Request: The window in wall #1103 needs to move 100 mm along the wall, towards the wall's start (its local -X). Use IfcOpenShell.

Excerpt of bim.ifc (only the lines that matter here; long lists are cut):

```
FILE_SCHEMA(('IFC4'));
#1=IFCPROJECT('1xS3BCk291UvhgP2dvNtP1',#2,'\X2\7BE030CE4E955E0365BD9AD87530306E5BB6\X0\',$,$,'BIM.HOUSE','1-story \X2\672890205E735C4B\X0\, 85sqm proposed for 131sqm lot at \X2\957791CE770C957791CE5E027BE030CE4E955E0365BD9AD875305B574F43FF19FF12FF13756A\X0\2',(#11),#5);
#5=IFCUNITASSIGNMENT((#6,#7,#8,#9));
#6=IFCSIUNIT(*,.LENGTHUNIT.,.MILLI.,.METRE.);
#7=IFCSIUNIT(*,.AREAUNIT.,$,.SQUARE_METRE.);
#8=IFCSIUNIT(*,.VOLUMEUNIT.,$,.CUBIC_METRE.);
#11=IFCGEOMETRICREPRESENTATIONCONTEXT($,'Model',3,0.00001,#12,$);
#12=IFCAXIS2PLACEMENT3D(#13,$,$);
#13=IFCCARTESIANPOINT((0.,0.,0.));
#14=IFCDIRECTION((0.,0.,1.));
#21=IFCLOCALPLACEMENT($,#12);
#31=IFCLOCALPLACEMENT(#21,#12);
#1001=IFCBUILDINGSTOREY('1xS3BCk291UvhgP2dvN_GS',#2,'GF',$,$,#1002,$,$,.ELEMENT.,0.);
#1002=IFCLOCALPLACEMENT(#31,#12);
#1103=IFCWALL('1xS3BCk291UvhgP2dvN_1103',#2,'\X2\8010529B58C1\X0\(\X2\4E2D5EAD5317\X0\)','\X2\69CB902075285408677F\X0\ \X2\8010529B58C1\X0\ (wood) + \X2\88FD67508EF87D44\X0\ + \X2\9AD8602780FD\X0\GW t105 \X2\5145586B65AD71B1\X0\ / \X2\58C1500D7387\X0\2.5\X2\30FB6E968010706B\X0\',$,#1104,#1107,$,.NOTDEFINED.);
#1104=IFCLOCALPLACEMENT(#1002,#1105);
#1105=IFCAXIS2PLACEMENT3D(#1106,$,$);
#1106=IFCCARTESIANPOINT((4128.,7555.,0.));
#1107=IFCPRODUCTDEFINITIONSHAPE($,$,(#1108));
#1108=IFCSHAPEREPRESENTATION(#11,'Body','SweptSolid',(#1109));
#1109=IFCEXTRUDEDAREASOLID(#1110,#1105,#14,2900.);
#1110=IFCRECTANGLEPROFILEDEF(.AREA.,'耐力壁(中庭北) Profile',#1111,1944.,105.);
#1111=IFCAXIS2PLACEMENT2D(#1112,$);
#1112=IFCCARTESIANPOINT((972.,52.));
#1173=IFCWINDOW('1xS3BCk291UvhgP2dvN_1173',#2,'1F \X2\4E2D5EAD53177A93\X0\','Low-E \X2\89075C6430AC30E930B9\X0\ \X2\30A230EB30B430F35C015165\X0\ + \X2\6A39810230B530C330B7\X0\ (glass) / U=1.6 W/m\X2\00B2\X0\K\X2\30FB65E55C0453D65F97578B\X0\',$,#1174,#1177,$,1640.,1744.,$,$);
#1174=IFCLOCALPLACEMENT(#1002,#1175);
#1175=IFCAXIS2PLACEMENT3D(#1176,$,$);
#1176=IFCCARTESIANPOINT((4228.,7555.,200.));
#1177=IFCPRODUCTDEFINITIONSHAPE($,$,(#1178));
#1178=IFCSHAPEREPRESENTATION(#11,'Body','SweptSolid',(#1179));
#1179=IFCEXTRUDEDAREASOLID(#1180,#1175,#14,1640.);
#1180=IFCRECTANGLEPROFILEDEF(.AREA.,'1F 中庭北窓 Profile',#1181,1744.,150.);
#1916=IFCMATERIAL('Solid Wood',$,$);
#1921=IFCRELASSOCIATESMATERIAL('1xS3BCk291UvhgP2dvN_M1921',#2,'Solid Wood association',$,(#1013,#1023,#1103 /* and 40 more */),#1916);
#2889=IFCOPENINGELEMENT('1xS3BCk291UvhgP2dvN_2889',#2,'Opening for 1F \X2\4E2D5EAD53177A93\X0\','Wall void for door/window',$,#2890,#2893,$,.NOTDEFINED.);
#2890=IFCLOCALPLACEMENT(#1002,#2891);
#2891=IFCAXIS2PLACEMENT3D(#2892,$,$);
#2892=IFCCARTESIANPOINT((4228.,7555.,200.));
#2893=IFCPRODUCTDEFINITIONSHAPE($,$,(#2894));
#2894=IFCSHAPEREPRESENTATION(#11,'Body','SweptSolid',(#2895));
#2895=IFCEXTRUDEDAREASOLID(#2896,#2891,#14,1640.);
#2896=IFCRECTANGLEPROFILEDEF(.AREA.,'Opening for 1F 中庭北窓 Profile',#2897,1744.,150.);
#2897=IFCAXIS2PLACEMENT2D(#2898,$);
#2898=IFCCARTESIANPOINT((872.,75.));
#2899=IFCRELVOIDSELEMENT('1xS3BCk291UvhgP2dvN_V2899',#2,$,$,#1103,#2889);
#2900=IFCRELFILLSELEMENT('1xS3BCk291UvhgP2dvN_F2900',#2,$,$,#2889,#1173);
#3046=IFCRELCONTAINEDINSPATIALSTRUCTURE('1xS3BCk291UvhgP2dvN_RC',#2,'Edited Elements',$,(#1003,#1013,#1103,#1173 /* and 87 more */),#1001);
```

```python
import ifcopenshell
import ifcopenshell.api.geometry
import ifcopenshell.util.placement
import ifcopenshell.util.unit

model = ifcopenshell.open("bim.ifc")
unit_scale = ifcopenshell.util.unit.calculate_unit_scale(model)

window = model.by_guid("1xS3BCk291UvhgP2dvN_1173")
opening = window.FillsVoids[0].RelatingOpeningElement
wall = opening.VoidsElements[0].RelatingBuildingElement

wall_matrix = ifcopenshell.util.placement.get_local_placement(wall.ObjectPlacement)
shift = wall_matrix[:3, 0] * -0.1 / unit_scale
before = ifcopenshell.util.placement.get_local_placement(window.ObjectPlacement)[:3, 3].copy()

# The window is not placed relative to its opening, so move both.
for product in (opening, window):
    matrix = ifcopenshell.util.placement.get_local_placement(product.ObjectPlacement)
    matrix[:3, 3] += shift
    ifcopenshell.api.geometry.edit_object_placement(model, product=product, matrix=matrix, is_si=False)

after = ifcopenshell.util.placement.get_local_placement(window.ObjectPlacement)[:3, 3]
print("window moved by", (after - before).round(3) + 0.0)

model.write("bim-out.ifc")
```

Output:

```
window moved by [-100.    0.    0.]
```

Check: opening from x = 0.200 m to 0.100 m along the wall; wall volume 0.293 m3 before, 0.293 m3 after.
